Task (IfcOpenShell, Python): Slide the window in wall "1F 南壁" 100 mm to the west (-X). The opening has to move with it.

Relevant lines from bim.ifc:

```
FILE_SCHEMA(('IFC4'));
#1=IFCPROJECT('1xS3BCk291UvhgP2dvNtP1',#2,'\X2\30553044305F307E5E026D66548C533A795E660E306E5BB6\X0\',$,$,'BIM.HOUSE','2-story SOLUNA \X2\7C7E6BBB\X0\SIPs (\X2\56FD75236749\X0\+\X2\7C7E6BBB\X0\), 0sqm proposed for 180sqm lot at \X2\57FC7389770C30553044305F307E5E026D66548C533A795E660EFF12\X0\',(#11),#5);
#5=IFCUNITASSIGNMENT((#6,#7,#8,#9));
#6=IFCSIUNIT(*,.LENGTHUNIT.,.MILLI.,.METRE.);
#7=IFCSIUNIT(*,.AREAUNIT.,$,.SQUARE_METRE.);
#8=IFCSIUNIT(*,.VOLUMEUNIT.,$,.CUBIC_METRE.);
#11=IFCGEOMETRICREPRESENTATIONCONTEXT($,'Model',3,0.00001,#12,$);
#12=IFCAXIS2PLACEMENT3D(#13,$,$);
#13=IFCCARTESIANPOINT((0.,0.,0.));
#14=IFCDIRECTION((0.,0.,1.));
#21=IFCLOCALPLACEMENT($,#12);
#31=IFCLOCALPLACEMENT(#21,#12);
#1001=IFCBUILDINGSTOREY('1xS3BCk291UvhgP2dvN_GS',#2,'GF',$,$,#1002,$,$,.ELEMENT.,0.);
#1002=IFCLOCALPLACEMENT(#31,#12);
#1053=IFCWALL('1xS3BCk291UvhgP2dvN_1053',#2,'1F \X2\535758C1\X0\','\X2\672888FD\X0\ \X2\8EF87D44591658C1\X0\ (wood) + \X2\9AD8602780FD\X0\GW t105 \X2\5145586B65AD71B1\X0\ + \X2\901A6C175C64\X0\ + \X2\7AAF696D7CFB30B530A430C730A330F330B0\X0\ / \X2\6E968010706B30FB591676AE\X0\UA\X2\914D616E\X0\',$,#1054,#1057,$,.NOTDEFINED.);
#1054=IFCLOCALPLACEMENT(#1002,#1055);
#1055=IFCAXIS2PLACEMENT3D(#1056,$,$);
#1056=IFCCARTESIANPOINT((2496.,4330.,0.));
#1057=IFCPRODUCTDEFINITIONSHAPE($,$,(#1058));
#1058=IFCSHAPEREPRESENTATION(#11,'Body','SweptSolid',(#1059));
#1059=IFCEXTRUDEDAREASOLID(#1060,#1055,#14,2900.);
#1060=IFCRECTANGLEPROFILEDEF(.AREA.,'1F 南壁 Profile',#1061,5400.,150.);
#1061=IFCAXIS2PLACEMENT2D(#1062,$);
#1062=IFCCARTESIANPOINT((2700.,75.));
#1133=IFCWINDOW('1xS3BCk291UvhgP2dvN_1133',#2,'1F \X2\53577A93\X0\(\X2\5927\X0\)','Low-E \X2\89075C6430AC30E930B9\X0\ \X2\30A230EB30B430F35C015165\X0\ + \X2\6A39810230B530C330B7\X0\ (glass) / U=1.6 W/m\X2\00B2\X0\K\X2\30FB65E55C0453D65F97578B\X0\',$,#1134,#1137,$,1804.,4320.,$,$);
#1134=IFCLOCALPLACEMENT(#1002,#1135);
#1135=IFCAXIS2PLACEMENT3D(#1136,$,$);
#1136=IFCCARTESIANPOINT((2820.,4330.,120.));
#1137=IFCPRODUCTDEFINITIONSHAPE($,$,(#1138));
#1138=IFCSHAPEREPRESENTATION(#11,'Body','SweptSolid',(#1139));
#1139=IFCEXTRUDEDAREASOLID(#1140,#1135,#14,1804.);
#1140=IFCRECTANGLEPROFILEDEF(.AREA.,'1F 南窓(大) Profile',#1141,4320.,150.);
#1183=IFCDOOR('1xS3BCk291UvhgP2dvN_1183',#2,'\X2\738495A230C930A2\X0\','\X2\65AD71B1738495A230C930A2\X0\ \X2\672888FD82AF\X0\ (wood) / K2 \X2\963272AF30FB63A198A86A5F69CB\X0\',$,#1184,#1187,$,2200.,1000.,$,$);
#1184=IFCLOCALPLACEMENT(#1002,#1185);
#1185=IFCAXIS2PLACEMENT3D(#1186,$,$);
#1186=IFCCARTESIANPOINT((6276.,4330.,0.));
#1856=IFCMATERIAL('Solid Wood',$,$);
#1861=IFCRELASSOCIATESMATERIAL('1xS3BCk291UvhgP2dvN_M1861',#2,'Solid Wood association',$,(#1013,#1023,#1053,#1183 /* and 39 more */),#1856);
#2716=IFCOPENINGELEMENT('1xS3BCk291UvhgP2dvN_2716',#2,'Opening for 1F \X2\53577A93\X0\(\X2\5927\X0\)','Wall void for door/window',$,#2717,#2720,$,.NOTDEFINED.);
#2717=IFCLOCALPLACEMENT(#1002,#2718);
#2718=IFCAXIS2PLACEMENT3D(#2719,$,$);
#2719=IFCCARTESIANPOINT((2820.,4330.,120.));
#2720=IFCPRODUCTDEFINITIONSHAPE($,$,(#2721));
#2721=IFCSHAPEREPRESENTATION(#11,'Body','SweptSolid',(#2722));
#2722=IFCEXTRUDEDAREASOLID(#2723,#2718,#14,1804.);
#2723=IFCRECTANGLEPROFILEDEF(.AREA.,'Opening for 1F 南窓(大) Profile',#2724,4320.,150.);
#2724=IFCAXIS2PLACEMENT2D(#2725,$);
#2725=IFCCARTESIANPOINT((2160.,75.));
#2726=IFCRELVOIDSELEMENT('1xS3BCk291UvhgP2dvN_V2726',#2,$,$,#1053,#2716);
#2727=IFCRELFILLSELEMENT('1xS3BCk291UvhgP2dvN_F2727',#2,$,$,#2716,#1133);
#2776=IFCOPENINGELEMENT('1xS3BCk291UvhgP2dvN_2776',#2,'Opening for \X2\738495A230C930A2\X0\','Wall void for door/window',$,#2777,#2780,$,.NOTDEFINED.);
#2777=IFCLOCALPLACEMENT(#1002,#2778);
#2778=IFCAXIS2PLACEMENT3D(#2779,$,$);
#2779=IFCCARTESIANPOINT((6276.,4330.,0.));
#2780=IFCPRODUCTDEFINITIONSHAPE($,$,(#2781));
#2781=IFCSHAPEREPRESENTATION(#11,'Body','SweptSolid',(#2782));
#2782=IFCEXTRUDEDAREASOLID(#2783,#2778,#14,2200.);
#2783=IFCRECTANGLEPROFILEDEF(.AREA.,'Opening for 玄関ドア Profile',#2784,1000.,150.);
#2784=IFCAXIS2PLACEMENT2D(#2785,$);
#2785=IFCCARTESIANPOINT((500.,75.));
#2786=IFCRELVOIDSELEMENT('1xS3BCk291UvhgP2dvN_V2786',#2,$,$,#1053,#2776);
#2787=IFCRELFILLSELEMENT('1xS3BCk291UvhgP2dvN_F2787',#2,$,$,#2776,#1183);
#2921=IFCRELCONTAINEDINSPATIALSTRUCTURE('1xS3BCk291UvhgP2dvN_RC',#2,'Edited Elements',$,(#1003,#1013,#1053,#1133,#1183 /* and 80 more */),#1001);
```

```python
import ifcopenshell
import ifcopenshell.api.geometry
import ifcopenshell.util.placement
import ifcopenshell.util.unit

model = ifcopenshell.open("bim.ifc")
unit_scale = ifcopenshell.util.unit.calculate_unit_scale(model)

window = model.by_guid("1xS3BCk291UvhgP2dvN_1133")
opening = window.FillsVoids[0].RelatingOpeningElement
wall = opening.VoidsElements[0].RelatingBuildingElement

wall_matrix = ifcopenshell.util.placement.get_local_placement(wall.ObjectPlacement)
shift = wall_matrix[:3, 0] * -0.1 / unit_scale
before = ifcopenshell.util.placement.get_local_placement(window.ObjectPlacement)[:3, 3].copy()

# The window is not placed relative to its opening, so move both.
for product in (opening, window):
    matrix = ifcopenshell.util.placement.get_local_placement(product.ObjectPlacement)
    matrix[:3, 3] += shift
    ifcopenshell.api.geometry.edit_object_placement(model, product=product, matrix=matrix, is_si=False)

after = ifcopenshell.util.placement.get_local_placement(window.ObjectPlacement)[:3, 3]
print("window moved by", (after - before).round(3) + 0.0)

model.write("bim_updated.ifc")
```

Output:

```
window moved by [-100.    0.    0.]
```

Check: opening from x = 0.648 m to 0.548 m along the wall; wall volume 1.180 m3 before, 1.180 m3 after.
